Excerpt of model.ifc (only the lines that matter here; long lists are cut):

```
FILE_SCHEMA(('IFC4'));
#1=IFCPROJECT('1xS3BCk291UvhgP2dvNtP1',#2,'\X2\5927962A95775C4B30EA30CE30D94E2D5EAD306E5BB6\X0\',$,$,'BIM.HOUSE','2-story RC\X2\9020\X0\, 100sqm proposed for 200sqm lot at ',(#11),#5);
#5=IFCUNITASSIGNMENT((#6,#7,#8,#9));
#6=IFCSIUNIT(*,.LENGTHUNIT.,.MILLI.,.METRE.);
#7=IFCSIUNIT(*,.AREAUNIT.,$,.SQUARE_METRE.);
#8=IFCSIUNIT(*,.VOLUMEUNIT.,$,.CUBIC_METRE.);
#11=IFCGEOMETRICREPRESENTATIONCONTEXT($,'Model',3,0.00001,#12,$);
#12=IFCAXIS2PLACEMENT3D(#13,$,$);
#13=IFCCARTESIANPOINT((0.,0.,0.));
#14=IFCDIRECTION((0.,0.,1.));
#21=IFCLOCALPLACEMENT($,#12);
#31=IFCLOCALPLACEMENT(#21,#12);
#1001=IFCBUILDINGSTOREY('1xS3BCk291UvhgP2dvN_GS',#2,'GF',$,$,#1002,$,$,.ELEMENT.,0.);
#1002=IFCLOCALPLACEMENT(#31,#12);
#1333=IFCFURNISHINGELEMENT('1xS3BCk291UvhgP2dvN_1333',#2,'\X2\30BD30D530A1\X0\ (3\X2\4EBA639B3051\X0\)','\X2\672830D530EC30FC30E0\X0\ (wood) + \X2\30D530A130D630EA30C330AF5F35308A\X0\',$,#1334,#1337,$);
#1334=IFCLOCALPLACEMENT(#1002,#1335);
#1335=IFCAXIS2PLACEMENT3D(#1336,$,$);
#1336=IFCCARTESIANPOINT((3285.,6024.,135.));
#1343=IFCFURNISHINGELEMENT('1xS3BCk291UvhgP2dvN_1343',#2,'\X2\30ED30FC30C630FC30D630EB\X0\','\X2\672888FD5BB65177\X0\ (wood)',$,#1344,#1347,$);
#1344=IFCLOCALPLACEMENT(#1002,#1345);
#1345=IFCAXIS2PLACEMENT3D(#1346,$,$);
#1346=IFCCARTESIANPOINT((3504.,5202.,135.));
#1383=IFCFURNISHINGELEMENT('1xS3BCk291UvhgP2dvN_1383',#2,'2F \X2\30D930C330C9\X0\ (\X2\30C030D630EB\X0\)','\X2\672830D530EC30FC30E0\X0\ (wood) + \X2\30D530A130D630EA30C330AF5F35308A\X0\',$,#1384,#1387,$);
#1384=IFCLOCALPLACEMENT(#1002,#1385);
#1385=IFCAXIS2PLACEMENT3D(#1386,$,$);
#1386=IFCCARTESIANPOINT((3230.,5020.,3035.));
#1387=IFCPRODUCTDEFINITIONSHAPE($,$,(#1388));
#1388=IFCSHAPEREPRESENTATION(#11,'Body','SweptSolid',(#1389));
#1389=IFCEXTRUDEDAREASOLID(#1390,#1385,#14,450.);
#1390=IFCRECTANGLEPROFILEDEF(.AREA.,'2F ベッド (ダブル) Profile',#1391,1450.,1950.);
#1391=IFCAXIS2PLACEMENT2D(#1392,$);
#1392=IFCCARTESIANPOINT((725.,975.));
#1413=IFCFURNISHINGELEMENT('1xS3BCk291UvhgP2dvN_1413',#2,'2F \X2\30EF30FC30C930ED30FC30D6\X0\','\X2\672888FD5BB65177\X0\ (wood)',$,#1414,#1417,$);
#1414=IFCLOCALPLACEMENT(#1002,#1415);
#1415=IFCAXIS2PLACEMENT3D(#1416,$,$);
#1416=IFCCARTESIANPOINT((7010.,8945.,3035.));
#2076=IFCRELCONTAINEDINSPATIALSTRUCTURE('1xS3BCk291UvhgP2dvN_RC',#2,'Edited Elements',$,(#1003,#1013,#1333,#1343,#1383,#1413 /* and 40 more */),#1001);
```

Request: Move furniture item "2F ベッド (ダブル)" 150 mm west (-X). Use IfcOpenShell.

```python
import ifcopenshell
import ifcopenshell.api.geometry
import ifcopenshell.util.placement

model = ifcopenshell.open("model.ifc")

item = model.by_guid("1xS3BCk291UvhgP2dvN_1383")
matrix = ifcopenshell.util.placement.get_local_placement(item.ObjectPlacement)
matrix[0, 3] -= 150.0
ifcopenshell.api.geometry.edit_object_placement(model, product=item, matrix=matrix, is_si=False)

print(ifcopenshell.util.placement.get_local_placement(item.ObjectPlacement).round(3) + 0.0)

model.write("model_updated.ifc")
```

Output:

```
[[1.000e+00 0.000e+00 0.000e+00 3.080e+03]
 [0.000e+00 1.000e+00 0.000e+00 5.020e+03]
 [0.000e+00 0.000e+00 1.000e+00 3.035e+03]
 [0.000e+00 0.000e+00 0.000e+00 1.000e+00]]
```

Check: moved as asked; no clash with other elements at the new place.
